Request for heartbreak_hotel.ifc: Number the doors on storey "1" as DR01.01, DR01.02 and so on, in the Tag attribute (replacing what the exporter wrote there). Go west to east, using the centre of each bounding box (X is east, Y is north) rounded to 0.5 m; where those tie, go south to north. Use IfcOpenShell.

First a look at what the model holds.

```python
import ifcopenshell
import ifcopenshell.util.element
import ifcopenshell.util.placement

model = ifcopenshell.open("heartbreak_hotel.ifc")
print(model.schema)
storey = next(s for s in model.by_type("IfcBuildingStorey") if s.Name == "1")
doors = [e for e in ifcopenshell.util.element.get_decomposition(storey) if e.is_a("IfcDoor")]
for e in sorted(doors, key=lambda e: e.id()):
    origin = ifcopenshell.util.placement.get_local_placement(e.ObjectPlacement)[:3, 3]
    print(e.id(), e.Tag, e.Name, origin.round(2) + 0.0, sep=" | ")
```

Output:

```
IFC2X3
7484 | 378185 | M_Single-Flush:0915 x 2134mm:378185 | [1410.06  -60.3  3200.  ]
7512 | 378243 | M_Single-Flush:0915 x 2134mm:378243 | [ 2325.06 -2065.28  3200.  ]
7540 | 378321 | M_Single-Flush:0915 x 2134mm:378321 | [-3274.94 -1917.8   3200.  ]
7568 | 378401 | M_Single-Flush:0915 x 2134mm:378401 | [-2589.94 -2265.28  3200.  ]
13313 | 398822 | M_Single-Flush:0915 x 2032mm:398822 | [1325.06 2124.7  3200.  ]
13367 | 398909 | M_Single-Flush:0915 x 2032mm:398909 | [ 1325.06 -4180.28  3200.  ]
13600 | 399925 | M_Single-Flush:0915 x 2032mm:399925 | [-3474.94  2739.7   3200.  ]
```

```python
import ifcopenshell
import ifcopenshell.geom
import ifcopenshell.util.element
import ifcopenshell.util.shape

model = ifcopenshell.open("heartbreak_hotel.ifc")
settings = ifcopenshell.geom.settings()
settings.set("use-world-coords", True)


def centre(element):
    shape = ifcopenshell.geom.create_shape(settings, element)
    return ifcopenshell.util.shape.get_bbox_centroid(shape.geometry)


storey = next(s for s in model.by_type("IfcBuildingStorey") if s.Name == "1")
doors = [e for e in ifcopenshell.util.element.get_decomposition(storey) if e.is_a("IfcDoor")]

# Insertion points can sit at a corner or the storey origin, so sort by the geometry (in metres).
centres = {e: centre(e) for e in doors}
doors.sort(key=lambda e: (round(centres[e][0] / 0.5), centres[e][1]))

for i, e in enumerate(doors, start=1):
    number = f"DR01.{i:02d}"
    e.Tag = number
    print(e.id(), number)

model.write("heartbreak_hotel-out.ifc")
```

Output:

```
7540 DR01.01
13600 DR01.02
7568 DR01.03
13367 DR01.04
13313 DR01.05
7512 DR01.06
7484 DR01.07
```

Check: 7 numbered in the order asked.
